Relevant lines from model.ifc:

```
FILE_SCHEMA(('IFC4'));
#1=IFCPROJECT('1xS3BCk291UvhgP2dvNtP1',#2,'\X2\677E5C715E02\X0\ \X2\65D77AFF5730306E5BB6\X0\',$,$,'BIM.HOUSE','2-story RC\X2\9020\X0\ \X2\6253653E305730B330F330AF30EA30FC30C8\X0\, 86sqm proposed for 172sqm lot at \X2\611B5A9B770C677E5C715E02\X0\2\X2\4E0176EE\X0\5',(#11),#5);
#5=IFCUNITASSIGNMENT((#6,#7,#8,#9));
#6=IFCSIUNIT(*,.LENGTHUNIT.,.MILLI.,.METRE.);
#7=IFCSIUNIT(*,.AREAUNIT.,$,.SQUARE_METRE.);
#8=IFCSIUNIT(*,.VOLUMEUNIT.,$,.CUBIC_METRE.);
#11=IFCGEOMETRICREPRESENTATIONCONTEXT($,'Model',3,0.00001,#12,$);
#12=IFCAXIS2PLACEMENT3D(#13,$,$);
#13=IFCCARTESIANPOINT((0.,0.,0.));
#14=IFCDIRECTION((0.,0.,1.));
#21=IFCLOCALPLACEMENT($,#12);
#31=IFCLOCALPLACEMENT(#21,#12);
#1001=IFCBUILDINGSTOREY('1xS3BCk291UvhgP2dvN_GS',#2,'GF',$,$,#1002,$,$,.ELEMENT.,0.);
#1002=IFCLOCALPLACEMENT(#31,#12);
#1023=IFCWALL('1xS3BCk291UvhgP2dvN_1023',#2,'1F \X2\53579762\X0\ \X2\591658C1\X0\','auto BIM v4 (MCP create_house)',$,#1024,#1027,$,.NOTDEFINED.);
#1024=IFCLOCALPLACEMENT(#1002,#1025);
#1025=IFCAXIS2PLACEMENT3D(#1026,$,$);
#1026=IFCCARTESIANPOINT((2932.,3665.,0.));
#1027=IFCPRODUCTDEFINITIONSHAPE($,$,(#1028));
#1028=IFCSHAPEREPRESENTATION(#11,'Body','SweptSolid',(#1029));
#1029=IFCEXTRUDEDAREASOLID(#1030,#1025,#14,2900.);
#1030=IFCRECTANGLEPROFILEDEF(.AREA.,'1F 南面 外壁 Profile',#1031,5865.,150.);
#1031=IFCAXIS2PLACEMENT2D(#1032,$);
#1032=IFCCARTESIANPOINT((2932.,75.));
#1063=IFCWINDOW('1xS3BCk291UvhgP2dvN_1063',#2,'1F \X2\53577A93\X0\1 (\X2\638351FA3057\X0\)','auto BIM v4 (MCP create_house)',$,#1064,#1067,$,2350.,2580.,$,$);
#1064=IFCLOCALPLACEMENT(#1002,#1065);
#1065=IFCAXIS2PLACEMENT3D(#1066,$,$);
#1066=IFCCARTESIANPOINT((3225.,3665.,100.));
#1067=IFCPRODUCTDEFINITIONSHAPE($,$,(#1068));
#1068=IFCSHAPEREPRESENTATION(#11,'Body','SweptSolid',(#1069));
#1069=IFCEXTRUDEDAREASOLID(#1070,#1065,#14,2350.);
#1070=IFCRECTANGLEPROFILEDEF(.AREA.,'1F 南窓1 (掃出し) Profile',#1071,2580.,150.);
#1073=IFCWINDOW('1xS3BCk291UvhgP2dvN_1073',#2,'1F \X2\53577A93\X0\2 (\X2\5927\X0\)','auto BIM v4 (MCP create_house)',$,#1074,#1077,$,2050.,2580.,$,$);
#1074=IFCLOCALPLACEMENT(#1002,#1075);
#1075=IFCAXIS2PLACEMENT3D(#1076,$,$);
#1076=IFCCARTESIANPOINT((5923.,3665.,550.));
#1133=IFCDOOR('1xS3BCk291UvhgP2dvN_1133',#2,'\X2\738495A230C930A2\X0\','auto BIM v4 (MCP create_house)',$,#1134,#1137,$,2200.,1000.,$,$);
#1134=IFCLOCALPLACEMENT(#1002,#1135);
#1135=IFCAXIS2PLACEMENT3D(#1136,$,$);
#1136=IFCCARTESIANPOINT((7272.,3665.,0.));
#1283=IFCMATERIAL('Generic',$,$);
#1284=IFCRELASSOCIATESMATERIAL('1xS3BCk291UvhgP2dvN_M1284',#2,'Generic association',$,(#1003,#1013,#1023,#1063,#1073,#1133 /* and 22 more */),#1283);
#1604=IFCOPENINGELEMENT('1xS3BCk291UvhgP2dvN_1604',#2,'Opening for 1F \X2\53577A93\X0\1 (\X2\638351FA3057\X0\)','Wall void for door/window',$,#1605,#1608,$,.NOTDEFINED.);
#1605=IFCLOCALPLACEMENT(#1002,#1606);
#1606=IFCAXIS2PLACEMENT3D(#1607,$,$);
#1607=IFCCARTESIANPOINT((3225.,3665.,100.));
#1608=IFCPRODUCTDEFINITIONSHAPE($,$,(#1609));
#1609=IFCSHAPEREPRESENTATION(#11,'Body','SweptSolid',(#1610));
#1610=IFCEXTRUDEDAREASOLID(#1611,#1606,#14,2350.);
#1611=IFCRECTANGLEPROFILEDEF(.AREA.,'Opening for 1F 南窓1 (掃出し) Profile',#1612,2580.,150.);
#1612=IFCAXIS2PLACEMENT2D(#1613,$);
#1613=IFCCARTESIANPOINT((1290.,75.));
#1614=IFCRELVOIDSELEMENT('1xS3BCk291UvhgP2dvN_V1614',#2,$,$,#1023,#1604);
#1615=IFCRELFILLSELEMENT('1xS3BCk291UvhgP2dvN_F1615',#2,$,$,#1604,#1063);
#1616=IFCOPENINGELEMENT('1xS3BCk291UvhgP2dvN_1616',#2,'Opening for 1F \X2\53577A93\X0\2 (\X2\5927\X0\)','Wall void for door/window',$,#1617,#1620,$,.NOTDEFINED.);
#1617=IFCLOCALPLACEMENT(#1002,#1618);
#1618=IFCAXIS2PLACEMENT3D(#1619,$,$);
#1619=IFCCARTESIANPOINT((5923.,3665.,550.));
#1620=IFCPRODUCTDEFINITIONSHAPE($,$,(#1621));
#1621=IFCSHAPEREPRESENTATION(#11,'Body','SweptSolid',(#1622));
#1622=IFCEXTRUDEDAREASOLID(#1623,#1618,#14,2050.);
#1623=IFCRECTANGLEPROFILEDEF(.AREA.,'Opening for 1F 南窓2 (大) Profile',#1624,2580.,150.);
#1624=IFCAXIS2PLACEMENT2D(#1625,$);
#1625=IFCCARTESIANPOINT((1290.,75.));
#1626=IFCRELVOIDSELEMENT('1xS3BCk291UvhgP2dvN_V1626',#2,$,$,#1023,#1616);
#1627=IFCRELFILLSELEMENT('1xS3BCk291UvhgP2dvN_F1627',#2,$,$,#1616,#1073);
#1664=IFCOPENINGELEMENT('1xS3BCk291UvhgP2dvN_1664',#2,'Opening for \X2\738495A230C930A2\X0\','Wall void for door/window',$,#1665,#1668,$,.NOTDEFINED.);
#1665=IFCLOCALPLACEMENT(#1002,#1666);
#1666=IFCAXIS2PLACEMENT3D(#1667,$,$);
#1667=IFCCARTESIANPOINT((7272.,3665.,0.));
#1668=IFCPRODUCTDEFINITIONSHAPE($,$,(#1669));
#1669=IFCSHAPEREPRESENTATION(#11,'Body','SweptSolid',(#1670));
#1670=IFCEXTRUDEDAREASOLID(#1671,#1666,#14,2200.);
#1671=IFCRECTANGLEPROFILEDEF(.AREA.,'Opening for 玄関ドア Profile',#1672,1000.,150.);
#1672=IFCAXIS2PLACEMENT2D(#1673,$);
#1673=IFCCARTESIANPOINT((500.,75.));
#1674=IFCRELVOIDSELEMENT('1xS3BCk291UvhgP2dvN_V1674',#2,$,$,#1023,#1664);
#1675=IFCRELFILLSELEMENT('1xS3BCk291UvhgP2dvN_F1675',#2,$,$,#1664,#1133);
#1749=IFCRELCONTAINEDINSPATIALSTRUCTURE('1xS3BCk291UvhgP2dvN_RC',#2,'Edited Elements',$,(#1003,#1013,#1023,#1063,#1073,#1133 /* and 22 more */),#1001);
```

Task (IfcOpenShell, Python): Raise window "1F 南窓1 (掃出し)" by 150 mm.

```python
import numpy as np
import ifcopenshell
import ifcopenshell.api.geometry
import ifcopenshell.util.placement
import ifcopenshell.util.unit

model = ifcopenshell.open("model.ifc")
unit_scale = ifcopenshell.util.unit.calculate_unit_scale(model)

window = model.by_guid("1xS3BCk291UvhgP2dvN_1063")
opening = window.FillsVoids[0].RelatingOpeningElement
dz = 150.0

shift = np.array([0.0, 0.0, dz])
# The window is not placed relative to its opening, so move both.
for product in (opening, window):
    matrix = ifcopenshell.util.placement.get_local_placement(product.ObjectPlacement)
    matrix[:3, 3] += shift
    ifcopenshell.api.geometry.edit_object_placement(model, product=product, matrix=matrix, is_si=False)

print(f"moved by {dz * unit_scale:+.3f} m")

model.write("model_edited.ifc")
```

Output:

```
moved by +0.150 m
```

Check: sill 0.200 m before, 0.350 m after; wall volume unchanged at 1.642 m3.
